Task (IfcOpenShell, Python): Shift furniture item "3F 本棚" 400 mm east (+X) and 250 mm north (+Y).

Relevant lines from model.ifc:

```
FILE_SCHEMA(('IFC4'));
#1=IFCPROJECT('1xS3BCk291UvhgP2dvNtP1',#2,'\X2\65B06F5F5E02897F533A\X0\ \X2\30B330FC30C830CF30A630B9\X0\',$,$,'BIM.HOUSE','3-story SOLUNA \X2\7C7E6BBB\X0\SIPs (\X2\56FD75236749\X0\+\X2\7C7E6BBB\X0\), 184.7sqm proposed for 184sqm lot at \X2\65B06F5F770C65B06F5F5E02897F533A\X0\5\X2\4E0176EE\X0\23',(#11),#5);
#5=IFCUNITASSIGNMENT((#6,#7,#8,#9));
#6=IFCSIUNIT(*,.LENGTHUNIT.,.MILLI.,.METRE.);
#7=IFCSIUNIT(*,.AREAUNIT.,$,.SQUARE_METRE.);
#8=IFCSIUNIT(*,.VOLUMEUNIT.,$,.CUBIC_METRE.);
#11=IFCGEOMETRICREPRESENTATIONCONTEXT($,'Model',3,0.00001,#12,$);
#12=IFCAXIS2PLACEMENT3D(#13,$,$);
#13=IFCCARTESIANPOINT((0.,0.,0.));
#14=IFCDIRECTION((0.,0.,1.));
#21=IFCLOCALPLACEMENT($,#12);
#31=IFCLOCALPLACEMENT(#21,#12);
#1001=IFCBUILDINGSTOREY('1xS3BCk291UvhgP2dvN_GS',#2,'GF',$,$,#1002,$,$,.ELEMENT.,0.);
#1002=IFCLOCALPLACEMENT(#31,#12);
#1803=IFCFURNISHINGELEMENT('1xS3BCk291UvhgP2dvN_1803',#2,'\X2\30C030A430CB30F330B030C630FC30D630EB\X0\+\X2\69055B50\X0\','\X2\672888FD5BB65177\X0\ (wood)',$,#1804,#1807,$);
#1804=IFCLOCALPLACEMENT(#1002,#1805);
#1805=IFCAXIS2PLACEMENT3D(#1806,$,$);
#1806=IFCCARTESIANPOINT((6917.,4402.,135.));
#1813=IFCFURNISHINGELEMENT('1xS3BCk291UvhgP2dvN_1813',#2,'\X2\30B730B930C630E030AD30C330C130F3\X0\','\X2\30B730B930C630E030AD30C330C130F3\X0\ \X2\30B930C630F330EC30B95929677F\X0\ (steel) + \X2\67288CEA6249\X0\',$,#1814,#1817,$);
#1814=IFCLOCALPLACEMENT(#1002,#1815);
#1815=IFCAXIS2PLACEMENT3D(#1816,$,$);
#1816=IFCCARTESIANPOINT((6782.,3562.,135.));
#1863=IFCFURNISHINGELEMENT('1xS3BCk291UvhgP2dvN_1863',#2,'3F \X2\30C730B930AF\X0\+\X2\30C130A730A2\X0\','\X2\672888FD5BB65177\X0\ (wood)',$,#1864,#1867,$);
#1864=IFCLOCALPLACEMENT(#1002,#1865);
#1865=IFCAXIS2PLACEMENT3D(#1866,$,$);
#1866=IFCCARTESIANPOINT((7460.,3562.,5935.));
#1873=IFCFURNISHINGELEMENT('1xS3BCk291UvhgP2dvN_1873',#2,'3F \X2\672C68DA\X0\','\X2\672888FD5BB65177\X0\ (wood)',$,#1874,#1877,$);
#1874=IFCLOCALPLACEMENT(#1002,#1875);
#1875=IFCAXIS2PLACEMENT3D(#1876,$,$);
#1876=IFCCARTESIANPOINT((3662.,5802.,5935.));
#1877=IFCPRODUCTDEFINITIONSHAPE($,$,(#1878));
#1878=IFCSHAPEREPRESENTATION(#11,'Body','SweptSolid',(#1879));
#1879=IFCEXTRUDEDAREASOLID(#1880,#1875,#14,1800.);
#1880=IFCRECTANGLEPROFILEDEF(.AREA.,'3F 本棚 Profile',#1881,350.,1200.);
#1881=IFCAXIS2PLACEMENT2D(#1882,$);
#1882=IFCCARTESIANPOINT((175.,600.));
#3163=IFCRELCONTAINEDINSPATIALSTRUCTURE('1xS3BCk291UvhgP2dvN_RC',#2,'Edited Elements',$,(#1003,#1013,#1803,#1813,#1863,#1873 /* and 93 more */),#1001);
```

```python
import ifcopenshell
import ifcopenshell.api.geometry
import ifcopenshell.util.placement

model = ifcopenshell.open("model.ifc")

item = model.by_id(1873)
matrix = ifcopenshell.util.placement.get_local_placement(item.ObjectPlacement)
matrix[0, 3] += 400.0
matrix[1, 3] += 250.0
ifcopenshell.api.geometry.edit_object_placement(model, product=item, matrix=matrix, is_si=False)

print(ifcopenshell.util.placement.get_local_placement(item.ObjectPlacement).round(3) + 0.0)

model.write("model_v2.ifc")
```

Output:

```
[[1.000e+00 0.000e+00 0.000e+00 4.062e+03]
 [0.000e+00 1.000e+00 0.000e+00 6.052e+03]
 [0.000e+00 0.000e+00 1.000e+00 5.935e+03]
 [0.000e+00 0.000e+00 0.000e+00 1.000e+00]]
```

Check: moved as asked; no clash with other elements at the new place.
